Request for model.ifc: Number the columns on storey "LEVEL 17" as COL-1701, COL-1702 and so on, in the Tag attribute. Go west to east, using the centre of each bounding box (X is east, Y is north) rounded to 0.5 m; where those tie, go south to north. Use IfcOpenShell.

First a look at what the model holds.

```python
import ifcopenshell
import ifcopenshell.util.element
import ifcopenshell.util.placement

model = ifcopenshell.open("model.ifc")
print(model.schema)
storey = next(s for s in model.by_type("IfcBuildingStorey") if s.Name == "LEVEL 17")
columns = [e for e in ifcopenshell.util.element.get_decomposition(storey) if e.is_a("IfcColumn")]
for e in sorted(columns, key=lambda e: e.id()):
    origin = ifcopenshell.util.placement.get_local_placement(e.ObjectPlacement)[:3, 3]
    print(e.id(), e.Tag, e.Name, origin.round(2) + 0.0, sep=" | ")
```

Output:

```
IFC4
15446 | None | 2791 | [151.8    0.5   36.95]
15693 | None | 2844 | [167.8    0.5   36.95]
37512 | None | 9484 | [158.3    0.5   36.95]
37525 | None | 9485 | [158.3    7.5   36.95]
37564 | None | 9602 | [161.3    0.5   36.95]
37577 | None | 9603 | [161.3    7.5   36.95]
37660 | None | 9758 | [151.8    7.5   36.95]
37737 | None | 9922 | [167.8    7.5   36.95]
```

```python
import ifcopenshell
import ifcopenshell.geom
import ifcopenshell.util.element
import ifcopenshell.util.shape

model = ifcopenshell.open("model.ifc")
settings = ifcopenshell.geom.settings()
settings.set("use-world-coords", True)


def centre(element):
    shape = ifcopenshell.geom.create_shape(settings, element)
    return ifcopenshell.util.shape.get_bbox_centroid(shape.geometry)


storey = next(s for s in model.by_type("IfcBuildingStorey") if s.Name == "LEVEL 17")
columns = [e for e in ifcopenshell.util.element.get_decomposition(storey) if e.is_a("IfcColumn")]

# Insertion points can sit at a corner or the storey origin, so sort by the geometry (in metres).
centres = {e: centre(e) for e in columns}
columns.sort(key=lambda e: (round(centres[e][0] / 0.5), centres[e][1]))

for i, e in enumerate(columns, start=1):
    number = f"COL-17{i:02d}"
    e.Tag = number
    print(e.id(), number)

model.write("model-out.ifc")
```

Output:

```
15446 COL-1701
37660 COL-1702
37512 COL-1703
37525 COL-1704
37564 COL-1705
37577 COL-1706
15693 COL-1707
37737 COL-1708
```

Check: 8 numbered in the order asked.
